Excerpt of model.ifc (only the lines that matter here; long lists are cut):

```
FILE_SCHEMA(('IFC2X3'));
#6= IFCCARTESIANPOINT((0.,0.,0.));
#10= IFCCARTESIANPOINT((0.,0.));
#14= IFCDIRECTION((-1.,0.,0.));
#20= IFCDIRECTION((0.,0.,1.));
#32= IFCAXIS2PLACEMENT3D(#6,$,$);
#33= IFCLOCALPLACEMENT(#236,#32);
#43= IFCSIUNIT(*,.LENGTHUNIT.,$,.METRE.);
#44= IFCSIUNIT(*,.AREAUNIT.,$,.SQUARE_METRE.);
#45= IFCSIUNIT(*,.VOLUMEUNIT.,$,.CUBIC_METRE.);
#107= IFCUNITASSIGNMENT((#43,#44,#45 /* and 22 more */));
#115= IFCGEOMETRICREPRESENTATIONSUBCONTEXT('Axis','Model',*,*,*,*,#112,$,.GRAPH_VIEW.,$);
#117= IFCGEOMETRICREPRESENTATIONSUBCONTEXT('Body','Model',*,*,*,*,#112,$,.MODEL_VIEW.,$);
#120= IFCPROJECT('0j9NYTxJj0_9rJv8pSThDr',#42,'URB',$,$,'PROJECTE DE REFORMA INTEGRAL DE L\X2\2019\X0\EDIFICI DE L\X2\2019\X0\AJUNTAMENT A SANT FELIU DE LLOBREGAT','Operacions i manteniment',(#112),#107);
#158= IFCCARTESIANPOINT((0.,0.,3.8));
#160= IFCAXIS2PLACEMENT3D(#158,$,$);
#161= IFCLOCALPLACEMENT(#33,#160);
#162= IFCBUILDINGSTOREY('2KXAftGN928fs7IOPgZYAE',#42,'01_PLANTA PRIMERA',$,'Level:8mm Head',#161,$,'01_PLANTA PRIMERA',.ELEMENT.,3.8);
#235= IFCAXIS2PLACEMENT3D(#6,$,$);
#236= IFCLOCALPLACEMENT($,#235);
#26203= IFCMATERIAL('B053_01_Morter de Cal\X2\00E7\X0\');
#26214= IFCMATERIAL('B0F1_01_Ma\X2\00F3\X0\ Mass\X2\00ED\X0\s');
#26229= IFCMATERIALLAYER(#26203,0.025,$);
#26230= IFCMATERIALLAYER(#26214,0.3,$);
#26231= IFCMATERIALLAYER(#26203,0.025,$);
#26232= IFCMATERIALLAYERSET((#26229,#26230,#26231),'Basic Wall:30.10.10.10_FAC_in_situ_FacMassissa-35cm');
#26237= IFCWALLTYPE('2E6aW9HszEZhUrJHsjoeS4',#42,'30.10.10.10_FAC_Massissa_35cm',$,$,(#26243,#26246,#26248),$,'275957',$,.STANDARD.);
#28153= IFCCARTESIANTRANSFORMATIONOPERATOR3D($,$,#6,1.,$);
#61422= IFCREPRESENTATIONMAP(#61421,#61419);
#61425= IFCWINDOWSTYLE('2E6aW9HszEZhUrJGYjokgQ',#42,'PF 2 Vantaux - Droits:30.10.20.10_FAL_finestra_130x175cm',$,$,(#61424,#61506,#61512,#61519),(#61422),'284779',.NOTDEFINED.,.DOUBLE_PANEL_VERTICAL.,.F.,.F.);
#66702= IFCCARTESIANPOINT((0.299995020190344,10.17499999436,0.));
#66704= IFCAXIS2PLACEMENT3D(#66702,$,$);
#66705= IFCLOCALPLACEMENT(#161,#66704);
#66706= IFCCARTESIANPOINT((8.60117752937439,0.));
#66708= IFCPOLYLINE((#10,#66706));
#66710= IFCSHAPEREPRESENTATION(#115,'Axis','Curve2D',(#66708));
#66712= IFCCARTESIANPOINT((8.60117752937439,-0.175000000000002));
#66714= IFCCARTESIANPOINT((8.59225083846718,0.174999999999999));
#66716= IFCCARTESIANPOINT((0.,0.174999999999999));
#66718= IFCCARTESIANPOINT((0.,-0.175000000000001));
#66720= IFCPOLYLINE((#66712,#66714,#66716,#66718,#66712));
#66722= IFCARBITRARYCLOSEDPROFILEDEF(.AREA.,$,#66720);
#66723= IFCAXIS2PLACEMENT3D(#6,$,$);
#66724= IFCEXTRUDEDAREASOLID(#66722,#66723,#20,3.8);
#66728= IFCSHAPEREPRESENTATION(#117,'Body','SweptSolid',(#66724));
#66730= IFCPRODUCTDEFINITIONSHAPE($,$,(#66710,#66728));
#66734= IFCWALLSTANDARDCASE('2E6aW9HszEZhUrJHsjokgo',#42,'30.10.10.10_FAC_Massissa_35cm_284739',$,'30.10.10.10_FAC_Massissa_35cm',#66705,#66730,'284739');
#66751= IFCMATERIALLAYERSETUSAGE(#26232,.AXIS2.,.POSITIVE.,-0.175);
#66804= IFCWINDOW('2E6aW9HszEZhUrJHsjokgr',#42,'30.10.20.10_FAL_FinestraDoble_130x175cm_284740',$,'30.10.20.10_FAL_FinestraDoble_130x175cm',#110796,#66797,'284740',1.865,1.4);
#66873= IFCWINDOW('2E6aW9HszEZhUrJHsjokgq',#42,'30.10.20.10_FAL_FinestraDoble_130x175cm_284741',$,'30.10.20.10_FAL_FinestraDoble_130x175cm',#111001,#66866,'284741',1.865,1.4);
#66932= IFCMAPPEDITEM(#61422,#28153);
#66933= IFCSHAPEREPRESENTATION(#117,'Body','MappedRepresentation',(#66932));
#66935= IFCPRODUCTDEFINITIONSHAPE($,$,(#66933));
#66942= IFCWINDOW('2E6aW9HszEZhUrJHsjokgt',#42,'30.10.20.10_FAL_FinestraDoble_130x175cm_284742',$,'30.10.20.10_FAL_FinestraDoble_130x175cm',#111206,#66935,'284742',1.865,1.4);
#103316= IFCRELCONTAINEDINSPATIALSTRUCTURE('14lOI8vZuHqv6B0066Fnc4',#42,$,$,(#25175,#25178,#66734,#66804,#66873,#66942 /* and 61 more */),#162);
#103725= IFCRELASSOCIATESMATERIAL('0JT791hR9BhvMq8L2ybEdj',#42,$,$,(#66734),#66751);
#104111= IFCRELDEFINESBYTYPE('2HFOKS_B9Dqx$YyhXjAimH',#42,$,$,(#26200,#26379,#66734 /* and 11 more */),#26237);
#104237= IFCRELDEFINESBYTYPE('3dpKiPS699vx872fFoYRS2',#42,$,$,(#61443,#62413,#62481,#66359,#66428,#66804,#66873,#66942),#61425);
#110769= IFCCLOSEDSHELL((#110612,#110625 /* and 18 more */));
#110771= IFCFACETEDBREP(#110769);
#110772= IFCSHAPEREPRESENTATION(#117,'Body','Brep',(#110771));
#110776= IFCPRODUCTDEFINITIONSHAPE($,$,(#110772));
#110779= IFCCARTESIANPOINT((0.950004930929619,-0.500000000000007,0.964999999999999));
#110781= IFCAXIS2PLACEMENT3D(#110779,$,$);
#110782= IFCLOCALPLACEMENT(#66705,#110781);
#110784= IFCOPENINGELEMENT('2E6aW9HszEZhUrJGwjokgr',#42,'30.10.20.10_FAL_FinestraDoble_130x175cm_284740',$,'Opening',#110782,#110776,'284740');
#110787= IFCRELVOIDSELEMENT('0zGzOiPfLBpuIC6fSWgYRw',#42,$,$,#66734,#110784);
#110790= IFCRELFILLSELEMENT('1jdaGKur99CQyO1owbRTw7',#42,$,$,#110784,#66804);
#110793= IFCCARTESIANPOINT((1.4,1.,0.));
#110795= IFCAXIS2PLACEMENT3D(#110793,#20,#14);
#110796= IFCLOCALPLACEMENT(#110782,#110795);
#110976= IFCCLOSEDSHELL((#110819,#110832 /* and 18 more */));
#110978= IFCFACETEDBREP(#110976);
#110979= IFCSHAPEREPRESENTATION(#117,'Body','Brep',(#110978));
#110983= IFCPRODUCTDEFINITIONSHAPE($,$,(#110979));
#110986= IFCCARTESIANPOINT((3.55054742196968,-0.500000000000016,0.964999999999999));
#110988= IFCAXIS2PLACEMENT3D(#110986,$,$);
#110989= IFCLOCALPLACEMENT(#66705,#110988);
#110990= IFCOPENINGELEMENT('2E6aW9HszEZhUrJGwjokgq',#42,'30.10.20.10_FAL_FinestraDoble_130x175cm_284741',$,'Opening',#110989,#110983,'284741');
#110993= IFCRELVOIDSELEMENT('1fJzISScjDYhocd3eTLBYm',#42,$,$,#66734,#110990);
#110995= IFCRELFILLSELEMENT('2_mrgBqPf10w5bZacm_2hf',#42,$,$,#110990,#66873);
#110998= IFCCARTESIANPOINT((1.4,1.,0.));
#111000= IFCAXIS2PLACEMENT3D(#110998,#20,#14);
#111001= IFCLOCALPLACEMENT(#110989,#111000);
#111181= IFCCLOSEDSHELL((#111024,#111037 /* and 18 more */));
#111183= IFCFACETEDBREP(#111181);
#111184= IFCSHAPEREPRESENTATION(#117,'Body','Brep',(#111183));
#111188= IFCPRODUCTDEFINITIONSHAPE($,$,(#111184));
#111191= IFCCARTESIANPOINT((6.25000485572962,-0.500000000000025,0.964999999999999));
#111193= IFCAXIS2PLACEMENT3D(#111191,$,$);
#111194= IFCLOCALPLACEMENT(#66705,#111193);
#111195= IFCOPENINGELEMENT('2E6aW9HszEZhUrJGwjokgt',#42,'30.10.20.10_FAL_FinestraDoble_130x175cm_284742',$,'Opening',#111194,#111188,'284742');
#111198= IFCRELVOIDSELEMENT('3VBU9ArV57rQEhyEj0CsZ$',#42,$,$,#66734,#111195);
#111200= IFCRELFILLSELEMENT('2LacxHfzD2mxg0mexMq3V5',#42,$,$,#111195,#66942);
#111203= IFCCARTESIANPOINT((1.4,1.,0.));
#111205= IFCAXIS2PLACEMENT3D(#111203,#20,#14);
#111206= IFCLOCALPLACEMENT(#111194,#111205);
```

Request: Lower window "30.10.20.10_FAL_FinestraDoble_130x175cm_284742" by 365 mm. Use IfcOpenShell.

```python
import numpy as np
import ifcopenshell
import ifcopenshell.api.geometry
import ifcopenshell.util.placement
import ifcopenshell.util.unit

model = ifcopenshell.open("model.ifc")
unit_scale = ifcopenshell.util.unit.calculate_unit_scale(model)

window = model.by_id(66942)
opening = window.FillsVoids[0].RelatingOpeningElement
dz = -0.365

shift = np.array([0.0, 0.0, dz])
# The window is placed relative to its opening, so it follows when the opening moves.
matrix = ifcopenshell.util.placement.get_local_placement(opening.ObjectPlacement)
matrix[:3, 3] += shift
ifcopenshell.api.geometry.edit_object_placement(
    model, product=opening, matrix=matrix, is_si=False, should_transform_children=True
)

print(f"moved by {dz * unit_scale:+.3f} m")

model.write("model_rev.ifc")
```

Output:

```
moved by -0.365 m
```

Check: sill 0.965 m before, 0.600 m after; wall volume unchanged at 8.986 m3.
